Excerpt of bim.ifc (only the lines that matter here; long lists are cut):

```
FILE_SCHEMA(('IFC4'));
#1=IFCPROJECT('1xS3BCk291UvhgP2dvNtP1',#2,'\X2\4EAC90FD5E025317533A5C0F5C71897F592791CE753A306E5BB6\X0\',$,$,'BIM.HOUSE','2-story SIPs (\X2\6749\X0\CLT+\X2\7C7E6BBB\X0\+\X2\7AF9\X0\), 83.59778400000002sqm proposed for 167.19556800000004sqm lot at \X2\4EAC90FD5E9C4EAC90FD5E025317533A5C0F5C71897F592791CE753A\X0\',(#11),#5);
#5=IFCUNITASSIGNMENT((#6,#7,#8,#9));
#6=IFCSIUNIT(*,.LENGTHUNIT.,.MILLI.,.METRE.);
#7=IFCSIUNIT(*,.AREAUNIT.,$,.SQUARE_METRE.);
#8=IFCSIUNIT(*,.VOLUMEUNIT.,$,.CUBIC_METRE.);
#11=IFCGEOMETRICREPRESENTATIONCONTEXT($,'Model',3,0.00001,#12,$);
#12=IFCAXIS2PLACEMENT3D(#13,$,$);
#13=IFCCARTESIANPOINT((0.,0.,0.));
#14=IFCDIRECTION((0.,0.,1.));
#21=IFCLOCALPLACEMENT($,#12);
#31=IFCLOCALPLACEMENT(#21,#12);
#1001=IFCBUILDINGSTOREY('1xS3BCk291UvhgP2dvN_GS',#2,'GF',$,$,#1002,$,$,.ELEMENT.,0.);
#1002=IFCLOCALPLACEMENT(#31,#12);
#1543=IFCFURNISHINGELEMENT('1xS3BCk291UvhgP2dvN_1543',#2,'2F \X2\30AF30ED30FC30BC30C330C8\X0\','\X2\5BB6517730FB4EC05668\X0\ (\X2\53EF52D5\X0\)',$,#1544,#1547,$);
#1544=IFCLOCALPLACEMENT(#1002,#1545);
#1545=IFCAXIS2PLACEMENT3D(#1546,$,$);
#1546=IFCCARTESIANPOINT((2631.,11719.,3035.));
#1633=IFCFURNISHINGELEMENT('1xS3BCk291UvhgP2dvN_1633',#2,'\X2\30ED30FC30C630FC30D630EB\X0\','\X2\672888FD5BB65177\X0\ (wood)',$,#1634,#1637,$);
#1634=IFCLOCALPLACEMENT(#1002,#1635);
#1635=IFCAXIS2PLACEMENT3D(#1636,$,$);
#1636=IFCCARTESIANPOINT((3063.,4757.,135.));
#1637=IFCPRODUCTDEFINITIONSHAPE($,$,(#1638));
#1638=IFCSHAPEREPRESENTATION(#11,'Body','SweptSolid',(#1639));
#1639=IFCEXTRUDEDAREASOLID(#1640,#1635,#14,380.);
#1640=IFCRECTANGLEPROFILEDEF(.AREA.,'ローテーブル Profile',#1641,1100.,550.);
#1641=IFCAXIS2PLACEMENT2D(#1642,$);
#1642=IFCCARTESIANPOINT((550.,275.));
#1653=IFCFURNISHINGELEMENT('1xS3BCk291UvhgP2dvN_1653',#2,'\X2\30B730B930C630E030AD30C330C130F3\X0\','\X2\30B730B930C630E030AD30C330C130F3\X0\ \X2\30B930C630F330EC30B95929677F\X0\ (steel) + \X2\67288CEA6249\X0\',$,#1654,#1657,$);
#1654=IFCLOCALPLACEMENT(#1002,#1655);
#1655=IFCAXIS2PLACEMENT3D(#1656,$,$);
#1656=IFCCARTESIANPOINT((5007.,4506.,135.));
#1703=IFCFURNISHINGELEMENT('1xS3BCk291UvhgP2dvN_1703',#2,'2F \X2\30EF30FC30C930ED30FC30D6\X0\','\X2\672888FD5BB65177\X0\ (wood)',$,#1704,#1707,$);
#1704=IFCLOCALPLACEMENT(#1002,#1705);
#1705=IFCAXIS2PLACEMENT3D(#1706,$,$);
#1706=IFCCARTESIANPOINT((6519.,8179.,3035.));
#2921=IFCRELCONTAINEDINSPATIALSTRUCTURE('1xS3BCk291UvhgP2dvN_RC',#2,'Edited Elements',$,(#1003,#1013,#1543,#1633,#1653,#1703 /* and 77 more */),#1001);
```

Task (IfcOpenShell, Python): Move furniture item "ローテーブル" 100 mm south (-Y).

```python
import ifcopenshell
import ifcopenshell.api.geometry
import ifcopenshell.util.placement
import ifcopenshell.util.unit

model = ifcopenshell.open("bim.ifc")
unit_scale = ifcopenshell.util.unit.calculate_unit_scale(model)

item = model.by_guid("1xS3BCk291UvhgP2dvN_1633")
matrix = ifcopenshell.util.placement.get_local_placement(item.ObjectPlacement)
matrix[1, 3] -= 0.1 / unit_scale
ifcopenshell.api.geometry.edit_object_placement(model, product=item, matrix=matrix, is_si=False)

print(ifcopenshell.util.placement.get_local_placement(item.ObjectPlacement).round(3) + 0.0)

model.write("bim_rev.ifc")
```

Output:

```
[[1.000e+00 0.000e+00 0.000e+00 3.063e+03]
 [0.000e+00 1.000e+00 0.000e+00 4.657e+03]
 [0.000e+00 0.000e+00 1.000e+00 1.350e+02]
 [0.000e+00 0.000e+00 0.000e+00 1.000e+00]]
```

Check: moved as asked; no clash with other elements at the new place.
